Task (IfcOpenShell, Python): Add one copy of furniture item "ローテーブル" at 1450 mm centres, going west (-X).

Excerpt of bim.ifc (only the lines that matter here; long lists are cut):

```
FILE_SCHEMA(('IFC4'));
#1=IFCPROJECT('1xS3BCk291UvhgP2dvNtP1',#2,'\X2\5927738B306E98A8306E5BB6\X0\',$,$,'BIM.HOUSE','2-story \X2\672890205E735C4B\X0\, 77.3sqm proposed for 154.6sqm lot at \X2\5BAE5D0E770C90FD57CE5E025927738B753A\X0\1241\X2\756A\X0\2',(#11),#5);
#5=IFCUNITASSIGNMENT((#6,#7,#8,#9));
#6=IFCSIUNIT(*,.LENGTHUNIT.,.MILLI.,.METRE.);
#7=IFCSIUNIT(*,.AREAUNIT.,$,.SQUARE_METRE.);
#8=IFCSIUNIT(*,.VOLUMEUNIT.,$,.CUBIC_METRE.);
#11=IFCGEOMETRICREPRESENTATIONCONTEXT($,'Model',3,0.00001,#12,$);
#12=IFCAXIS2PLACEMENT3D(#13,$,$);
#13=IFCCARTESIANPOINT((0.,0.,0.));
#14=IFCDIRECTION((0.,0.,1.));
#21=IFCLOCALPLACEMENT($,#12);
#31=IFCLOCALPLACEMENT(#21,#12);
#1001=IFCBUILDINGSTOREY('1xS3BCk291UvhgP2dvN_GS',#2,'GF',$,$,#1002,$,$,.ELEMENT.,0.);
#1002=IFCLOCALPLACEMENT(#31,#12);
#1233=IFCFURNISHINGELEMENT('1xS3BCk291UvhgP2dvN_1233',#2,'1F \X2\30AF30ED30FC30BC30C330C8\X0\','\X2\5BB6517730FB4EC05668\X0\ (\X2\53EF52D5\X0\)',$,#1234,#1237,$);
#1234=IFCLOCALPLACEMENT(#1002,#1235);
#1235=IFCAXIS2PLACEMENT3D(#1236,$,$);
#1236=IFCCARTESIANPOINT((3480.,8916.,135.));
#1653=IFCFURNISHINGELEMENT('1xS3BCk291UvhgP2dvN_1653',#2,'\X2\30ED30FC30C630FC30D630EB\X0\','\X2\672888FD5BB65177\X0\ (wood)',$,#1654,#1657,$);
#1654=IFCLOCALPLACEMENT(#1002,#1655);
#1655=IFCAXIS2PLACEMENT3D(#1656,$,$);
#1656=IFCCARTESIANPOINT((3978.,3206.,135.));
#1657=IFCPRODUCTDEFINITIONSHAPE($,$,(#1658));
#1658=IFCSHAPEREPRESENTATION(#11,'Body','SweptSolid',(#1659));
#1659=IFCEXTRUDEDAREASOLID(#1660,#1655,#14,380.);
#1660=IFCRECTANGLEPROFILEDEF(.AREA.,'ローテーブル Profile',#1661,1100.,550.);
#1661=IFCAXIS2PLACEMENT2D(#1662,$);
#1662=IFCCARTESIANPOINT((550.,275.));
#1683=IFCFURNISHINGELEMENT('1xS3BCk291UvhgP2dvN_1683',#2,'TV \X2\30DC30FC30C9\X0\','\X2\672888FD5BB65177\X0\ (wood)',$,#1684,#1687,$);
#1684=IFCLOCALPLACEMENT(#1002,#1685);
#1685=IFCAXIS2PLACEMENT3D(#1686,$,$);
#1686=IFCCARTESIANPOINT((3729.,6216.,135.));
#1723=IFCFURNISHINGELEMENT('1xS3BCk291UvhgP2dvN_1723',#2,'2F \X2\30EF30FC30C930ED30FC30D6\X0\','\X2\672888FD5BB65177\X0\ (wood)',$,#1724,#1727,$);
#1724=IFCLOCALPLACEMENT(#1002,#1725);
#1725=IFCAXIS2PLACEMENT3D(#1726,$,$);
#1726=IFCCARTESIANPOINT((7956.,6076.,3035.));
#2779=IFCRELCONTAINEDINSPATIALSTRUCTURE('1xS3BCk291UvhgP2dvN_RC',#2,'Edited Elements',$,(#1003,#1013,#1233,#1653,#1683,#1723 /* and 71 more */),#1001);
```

```python
import numpy as np
import ifcopenshell
import ifcopenshell.api.geometry
import ifcopenshell.api.root
import ifcopenshell.util.element
import ifcopenshell.util.placement
import ifcopenshell.util.unit

model = ifcopenshell.open("bim.ifc")
unit_scale = ifcopenshell.util.unit.calculate_unit_scale(model)


def reuse_history(source, copy):
    """copy_class also copies each property set's owner history, people and application; keep the originals."""
    for rel in copy.IsDefinedBy:
        if rel.is_a("IfcRelDefinesByProperties") and (history := rel.RelatingPropertyDefinition.OwnerHistory):
            rel.RelatingPropertyDefinition.OwnerHistory = source.OwnerHistory
            ifcopenshell.util.element.remove_deep2(model, history)


source = model.by_id(1653)
base = ifcopenshell.util.placement.get_local_placement(source.ObjectPlacement)
step = np.array([-1.0, 0.0, 0.0]) * 1.45 / unit_scale

for i in range(1, 2):
    copy = ifcopenshell.api.root.copy_class(model, product=source)
    copy.Representation = ifcopenshell.util.element.copy_deep(
        model, source.Representation, exclude=["IfcGeometricRepresentationContext", "IfcRepresentationMap"]
    )
    reuse_history(source, copy)
    matrix = base.copy()
    matrix[:3, 3] += i * step
    print("added at", matrix[:3, 3].round(3) + 0.0)
    ifcopenshell.api.geometry.edit_object_placement(model, product=copy, matrix=matrix, is_si=False)

model.write("bim_rev.ifc")
```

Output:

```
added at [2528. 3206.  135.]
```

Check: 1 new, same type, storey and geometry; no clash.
